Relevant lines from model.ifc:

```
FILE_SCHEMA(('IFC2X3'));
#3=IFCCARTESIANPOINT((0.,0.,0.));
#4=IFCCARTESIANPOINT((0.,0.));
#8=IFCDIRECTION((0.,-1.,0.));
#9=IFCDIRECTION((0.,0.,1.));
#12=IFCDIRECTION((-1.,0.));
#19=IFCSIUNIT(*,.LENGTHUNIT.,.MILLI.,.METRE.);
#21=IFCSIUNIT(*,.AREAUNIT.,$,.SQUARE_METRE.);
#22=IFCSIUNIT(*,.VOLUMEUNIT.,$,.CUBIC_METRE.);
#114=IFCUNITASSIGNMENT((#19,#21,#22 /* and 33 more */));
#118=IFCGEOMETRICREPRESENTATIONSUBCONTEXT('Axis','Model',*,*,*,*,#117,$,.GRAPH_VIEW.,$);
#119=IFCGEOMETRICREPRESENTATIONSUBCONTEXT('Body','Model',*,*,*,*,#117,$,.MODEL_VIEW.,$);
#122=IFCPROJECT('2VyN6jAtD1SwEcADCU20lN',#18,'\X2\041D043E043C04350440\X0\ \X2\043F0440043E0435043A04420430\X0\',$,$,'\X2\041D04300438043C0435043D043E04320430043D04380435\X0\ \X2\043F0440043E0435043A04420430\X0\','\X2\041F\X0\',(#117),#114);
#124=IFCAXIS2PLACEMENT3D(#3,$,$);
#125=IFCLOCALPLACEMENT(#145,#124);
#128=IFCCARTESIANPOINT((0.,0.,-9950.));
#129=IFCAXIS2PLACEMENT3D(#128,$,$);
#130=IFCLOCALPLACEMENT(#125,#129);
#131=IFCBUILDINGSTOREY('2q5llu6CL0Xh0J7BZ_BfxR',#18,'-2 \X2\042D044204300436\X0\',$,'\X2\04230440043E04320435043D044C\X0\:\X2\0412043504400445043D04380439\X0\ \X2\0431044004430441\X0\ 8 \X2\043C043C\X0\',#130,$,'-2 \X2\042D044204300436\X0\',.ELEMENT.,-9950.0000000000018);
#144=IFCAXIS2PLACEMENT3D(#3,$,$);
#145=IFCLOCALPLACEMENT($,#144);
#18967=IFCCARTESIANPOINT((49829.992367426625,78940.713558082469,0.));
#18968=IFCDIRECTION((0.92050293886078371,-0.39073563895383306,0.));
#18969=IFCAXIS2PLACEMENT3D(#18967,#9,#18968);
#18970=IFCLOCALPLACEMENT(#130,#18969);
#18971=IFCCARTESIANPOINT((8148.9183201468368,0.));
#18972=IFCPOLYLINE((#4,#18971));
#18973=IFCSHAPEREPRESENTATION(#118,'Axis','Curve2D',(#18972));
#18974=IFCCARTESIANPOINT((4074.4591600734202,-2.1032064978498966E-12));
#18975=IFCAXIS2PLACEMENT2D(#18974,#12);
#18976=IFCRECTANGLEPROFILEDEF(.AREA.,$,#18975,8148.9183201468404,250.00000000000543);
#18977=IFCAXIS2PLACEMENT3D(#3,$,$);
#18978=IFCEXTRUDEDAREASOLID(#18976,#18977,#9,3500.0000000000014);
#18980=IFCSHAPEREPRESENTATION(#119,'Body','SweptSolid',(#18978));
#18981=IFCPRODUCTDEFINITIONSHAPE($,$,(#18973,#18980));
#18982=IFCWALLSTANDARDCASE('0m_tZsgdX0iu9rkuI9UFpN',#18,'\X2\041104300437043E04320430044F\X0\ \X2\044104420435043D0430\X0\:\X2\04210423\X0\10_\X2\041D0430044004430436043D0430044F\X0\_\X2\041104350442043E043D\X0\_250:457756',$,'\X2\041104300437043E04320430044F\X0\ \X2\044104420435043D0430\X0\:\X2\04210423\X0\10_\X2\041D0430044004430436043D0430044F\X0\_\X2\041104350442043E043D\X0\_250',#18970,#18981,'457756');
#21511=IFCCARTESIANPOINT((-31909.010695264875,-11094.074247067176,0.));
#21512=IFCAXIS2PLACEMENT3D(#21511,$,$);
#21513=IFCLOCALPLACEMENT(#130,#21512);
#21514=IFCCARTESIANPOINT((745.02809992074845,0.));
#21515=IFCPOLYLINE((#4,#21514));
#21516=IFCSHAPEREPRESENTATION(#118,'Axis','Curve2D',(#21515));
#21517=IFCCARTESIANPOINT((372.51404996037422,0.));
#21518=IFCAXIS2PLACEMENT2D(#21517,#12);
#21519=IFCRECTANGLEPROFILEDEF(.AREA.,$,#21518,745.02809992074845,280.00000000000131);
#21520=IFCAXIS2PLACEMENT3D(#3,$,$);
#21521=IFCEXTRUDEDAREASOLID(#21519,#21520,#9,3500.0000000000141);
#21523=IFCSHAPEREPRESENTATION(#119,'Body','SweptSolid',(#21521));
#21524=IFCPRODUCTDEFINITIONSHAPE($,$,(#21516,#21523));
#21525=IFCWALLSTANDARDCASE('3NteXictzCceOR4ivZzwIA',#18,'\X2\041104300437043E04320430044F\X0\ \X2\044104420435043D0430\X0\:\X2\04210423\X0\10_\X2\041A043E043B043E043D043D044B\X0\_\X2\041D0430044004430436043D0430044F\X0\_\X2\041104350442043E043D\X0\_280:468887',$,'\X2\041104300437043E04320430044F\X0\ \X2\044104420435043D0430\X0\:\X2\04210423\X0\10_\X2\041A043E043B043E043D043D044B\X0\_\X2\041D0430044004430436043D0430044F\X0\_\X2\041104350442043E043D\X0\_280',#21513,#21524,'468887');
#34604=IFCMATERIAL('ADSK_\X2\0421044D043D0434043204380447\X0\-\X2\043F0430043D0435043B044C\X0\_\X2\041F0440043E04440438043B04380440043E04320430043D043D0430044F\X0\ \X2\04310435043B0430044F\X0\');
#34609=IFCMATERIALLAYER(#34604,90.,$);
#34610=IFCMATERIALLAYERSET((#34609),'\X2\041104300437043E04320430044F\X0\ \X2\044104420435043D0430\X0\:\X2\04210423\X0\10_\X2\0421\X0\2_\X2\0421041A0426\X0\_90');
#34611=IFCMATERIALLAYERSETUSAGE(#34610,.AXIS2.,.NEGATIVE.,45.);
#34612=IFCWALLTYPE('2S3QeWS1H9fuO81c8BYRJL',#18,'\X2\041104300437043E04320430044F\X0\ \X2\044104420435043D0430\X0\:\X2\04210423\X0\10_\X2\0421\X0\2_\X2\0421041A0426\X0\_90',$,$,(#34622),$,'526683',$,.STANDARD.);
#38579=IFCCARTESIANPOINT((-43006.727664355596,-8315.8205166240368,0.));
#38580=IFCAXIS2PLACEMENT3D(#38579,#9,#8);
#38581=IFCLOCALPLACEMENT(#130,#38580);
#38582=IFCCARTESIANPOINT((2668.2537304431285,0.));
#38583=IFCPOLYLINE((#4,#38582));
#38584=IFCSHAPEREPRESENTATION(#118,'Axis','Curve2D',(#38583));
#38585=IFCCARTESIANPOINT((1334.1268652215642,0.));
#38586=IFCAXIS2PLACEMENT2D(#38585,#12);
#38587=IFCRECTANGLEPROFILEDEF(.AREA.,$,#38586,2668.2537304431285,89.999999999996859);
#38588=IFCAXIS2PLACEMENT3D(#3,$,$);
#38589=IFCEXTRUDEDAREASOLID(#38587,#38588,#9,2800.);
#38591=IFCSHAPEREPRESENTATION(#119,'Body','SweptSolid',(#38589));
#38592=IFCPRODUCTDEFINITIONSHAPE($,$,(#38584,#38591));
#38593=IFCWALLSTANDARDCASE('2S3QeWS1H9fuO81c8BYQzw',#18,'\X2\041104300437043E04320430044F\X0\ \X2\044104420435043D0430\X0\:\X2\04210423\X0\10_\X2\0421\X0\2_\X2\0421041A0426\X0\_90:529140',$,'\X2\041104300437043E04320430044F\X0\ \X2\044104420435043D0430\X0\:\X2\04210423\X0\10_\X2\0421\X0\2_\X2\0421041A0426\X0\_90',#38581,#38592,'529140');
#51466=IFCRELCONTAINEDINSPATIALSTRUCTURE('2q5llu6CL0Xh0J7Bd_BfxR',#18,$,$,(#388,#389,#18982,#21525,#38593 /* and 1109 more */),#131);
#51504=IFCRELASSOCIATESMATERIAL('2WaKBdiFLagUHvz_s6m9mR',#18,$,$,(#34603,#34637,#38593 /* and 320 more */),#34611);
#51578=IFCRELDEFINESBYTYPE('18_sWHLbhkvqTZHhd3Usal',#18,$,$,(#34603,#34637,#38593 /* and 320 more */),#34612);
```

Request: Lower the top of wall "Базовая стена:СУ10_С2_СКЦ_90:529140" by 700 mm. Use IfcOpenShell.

```python
import ifcopenshell
import ifcopenshell.geom
import ifcopenshell.util.representation
import ifcopenshell.util.shape

model = ifcopenshell.open("model.ifc")
settings = ifcopenshell.geom.settings()


def volume(element):
    """Net volume in cubic metres, openings subtracted."""
    shape = ifcopenshell.geom.create_shape(settings, element)
    return ifcopenshell.util.shape.get_volume(shape.geometry)


wall = model.by_guid("2S3QeWS1H9fuO81c8BYQzw")
before = volume(wall)

body = ifcopenshell.util.representation.get_representation(wall, "Model", "Body")
solid = body.Items[0]
old_height = solid.Depth
solid.Depth -= 700.0
after = volume(wall)

print(f"height {old_height:g} -> {solid.Depth:g}, volume {before:.3f} -> {after:.3f} m3")

model.write("model_edited.ifc")
```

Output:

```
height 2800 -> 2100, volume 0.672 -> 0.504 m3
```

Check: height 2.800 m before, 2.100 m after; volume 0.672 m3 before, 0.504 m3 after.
